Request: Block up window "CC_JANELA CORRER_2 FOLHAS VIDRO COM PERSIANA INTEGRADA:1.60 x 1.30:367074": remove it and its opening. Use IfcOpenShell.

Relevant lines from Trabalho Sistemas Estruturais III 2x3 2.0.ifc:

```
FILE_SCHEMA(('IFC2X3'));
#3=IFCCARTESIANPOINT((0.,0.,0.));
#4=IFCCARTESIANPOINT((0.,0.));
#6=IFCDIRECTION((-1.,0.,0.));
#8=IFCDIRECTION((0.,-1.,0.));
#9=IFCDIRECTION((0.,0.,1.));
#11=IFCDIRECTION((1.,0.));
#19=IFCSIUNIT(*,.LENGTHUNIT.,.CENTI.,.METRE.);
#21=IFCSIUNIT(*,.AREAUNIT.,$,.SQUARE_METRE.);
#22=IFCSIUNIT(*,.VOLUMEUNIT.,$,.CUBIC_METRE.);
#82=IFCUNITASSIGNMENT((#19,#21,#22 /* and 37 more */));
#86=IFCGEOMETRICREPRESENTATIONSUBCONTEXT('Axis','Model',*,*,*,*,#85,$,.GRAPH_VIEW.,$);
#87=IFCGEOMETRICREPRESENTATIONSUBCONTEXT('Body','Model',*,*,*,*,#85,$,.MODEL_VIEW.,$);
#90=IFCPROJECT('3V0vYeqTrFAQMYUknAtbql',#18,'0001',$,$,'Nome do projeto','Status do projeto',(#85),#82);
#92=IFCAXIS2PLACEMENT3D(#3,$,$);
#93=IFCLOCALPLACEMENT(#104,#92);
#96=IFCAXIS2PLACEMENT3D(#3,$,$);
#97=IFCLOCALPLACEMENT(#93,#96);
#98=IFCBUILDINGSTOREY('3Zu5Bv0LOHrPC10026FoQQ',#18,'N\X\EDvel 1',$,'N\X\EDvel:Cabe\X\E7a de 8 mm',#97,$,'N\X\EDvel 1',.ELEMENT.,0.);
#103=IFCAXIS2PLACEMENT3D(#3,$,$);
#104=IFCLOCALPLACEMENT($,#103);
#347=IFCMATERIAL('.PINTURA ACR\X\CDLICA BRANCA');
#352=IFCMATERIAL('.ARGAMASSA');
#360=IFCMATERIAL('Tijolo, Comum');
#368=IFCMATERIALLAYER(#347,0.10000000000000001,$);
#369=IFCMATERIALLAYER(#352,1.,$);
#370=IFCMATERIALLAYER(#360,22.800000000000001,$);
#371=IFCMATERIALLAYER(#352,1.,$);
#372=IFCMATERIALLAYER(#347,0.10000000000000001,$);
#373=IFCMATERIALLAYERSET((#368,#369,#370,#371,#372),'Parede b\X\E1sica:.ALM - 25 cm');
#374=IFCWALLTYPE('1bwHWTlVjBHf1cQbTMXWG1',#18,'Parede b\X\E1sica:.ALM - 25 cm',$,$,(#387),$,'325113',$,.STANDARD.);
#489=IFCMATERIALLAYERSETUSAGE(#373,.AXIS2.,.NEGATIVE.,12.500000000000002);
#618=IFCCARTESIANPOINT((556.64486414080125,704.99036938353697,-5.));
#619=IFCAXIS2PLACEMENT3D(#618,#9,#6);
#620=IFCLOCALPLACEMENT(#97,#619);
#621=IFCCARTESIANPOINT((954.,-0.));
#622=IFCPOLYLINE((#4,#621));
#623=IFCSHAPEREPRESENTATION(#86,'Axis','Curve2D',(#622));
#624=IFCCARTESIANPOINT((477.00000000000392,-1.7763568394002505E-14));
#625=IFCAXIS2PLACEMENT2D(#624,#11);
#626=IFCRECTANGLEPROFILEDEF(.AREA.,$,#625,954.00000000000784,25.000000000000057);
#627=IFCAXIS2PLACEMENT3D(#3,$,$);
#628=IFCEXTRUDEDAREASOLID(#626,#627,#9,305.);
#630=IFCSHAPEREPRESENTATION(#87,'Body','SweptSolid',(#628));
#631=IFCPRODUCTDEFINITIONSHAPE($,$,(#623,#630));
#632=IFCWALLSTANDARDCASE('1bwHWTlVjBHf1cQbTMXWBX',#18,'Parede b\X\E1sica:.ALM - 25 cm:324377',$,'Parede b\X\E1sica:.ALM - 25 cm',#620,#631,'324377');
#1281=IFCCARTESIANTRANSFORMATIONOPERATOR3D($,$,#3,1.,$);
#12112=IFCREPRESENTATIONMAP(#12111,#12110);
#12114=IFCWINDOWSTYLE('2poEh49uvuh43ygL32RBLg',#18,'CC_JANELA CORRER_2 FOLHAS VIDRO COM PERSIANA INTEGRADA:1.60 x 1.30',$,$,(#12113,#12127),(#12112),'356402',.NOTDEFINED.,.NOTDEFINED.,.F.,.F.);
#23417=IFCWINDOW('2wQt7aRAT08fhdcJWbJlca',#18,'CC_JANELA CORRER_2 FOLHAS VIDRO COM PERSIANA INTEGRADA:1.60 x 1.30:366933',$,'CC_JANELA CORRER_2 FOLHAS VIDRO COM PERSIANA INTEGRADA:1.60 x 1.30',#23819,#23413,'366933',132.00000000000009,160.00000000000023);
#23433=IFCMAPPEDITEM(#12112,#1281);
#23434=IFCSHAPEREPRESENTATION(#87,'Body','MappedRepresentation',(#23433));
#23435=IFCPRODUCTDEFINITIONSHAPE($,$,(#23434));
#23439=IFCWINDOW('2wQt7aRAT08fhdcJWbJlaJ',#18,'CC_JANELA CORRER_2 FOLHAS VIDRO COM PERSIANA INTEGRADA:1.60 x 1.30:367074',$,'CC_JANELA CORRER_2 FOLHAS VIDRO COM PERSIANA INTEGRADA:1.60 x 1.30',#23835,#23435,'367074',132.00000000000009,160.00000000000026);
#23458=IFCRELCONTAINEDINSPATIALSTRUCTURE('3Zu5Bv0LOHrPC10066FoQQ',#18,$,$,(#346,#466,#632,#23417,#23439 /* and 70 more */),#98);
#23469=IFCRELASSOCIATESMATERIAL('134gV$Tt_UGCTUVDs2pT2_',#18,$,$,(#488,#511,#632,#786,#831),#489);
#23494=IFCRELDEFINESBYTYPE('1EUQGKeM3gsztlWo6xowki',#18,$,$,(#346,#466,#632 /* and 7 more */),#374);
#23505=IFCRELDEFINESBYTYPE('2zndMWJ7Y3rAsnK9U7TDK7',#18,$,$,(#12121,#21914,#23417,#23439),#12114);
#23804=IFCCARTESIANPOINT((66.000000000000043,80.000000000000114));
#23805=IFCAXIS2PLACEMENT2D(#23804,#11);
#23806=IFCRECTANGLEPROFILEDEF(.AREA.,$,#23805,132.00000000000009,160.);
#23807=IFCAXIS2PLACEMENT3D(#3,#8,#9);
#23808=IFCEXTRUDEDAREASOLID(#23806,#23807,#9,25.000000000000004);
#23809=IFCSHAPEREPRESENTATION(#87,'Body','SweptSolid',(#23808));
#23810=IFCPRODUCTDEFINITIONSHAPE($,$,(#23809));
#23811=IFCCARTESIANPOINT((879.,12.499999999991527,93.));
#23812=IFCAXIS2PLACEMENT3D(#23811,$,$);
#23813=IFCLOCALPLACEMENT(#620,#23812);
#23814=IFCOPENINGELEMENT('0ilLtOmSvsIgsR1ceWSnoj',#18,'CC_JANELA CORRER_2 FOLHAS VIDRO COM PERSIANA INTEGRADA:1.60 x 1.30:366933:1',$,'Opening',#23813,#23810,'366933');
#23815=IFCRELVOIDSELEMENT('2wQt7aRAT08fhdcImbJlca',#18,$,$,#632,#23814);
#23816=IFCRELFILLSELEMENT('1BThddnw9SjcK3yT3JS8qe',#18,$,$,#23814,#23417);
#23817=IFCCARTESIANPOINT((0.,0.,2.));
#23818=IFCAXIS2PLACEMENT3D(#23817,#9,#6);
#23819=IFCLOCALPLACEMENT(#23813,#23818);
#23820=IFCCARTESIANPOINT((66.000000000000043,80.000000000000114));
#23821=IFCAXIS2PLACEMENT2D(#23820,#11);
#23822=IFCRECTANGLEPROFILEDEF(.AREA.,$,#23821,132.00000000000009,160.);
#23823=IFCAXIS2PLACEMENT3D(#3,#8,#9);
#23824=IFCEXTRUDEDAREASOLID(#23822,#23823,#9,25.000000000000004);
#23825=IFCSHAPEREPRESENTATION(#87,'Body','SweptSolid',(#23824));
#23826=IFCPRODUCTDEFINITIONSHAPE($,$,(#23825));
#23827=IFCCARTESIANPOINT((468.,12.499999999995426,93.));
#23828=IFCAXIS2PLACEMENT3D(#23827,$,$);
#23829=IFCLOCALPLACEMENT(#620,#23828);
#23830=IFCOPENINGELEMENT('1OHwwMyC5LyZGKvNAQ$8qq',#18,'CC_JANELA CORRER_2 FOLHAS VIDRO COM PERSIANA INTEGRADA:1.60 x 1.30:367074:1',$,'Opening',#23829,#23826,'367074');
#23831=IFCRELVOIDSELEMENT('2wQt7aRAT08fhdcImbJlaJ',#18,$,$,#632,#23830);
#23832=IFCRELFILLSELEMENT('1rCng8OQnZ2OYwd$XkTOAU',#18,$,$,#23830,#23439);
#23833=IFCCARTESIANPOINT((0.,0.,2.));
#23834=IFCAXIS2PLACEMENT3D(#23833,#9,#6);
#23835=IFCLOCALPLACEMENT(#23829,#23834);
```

```python
import ifcopenshell
import ifcopenshell.api.feature
import ifcopenshell.api.root
import ifcopenshell.geom
import ifcopenshell.util.shape

model = ifcopenshell.open("Trabalho Sistemas Estruturais III 2x3 2.0.ifc")
settings = ifcopenshell.geom.settings()


def volume(element):
    """Net volume in cubic metres, openings subtracted."""
    shape = ifcopenshell.geom.create_shape(settings, element)
    return ifcopenshell.util.shape.get_volume(shape.geometry)


window = model.by_id(23439)
opening = window.FillsVoids[0].RelatingOpeningElement
wall = opening.VoidsElements[0].RelatingBuildingElement
before = volume(wall)

ifcopenshell.api.root.remove_product(model, product=window)
ifcopenshell.api.feature.remove_feature(model, feature=opening)

after = volume(wall)

print(f"wall volume {before:.3f} -> {after:.3f} m3")

model.write("Trabalho Sistemas Estruturais III 2x3 2.0_updated.ifc")
```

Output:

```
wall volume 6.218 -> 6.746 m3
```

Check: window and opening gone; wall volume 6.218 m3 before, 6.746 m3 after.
